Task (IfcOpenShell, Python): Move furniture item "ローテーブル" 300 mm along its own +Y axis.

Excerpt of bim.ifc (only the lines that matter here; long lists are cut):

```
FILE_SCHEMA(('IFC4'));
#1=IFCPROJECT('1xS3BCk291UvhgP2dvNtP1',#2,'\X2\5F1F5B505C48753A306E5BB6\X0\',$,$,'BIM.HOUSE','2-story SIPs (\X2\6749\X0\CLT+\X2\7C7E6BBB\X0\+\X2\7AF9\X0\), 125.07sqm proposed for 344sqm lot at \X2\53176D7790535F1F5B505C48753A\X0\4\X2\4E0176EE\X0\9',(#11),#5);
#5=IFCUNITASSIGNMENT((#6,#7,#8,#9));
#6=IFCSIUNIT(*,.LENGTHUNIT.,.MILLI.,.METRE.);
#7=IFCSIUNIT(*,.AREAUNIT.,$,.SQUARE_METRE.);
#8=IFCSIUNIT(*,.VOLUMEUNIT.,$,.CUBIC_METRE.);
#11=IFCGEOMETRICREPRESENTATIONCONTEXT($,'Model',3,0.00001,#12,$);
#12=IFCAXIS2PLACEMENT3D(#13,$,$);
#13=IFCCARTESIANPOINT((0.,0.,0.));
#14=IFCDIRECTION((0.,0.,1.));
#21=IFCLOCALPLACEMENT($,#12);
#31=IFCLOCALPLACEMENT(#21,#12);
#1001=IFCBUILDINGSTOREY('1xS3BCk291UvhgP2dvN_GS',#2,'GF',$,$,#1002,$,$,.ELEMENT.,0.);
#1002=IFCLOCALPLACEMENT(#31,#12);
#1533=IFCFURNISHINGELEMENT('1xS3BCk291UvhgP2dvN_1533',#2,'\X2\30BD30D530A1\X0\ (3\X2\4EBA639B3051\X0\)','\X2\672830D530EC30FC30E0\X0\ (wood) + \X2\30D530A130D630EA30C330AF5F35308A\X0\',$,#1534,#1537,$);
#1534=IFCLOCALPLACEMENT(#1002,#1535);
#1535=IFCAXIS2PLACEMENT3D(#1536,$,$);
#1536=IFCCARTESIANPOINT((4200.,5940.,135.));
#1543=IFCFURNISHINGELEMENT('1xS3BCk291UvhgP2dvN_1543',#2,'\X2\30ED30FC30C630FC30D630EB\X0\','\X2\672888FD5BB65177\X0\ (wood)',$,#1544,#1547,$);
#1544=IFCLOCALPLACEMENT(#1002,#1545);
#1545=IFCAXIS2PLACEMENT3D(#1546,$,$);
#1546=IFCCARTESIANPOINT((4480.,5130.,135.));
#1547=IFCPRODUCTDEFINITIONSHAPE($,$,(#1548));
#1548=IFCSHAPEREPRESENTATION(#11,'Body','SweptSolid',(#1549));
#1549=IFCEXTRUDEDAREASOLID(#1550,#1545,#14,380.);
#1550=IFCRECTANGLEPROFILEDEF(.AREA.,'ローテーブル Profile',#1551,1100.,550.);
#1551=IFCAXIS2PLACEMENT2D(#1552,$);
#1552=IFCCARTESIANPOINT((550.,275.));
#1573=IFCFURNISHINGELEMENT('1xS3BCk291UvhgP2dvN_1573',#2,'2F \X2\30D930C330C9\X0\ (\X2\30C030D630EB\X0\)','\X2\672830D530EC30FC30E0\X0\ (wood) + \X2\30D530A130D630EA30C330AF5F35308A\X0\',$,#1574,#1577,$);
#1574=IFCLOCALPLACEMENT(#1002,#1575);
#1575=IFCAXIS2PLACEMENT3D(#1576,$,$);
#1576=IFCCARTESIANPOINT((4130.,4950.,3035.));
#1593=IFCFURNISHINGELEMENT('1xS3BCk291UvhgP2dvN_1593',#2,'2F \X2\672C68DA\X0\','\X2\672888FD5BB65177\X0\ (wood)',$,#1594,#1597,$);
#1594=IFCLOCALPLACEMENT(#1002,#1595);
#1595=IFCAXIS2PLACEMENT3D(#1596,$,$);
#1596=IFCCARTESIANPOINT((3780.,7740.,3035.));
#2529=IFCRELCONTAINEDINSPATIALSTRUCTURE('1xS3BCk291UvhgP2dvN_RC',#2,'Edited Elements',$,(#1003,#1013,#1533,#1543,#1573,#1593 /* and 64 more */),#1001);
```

```python
import ifcopenshell
import ifcopenshell.api.geometry
import ifcopenshell.util.placement

model = ifcopenshell.open("bim.ifc")

item = model.by_guid("1xS3BCk291UvhgP2dvN_1543")
matrix = ifcopenshell.util.placement.get_local_placement(item.ObjectPlacement)
matrix[:3, 3] += matrix[:3, 1] * 300.0
ifcopenshell.api.geometry.edit_object_placement(model, product=item, matrix=matrix, is_si=False)

print(ifcopenshell.util.placement.get_local_placement(item.ObjectPlacement).round(3) + 0.0)

model.write("bim_v2.ifc")
```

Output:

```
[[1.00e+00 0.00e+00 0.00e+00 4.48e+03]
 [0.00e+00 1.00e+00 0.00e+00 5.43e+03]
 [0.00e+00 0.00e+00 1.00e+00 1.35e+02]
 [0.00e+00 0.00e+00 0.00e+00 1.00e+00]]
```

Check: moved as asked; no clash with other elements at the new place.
